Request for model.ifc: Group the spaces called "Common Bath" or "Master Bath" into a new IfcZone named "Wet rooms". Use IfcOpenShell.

First a look at what the model holds.

```python
import ifcopenshell

model = ifcopenshell.open("model.ifc")
print(model.schema)
seen = {}
for space in model.by_type("IfcSpace"):
    seen[space.LongName] = seen.get(space.LongName, 0) + 1
for name, count in sorted(seen.items(), key=str):
    print(count, "x", name)
print("zones:", [z.Name for z in model.by_type("IfcZone")][:20])
```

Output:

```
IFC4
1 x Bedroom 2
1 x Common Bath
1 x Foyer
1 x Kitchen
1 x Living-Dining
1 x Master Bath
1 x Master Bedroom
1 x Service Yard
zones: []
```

```python
import ifcopenshell
import ifcopenshell.api.group
import ifcopenshell.api.root

model = ifcopenshell.open("model.ifc")

names = {"Common Bath", "Master Bath"}
spaces = [s for s in model.by_type("IfcSpace") if s.LongName in names]

zone = ifcopenshell.api.root.create_entity(model, ifc_class="IfcZone", name="Wet rooms")
ifcopenshell.api.group.assign_group(model, products=spaces, group=zone)
print(len(spaces), "spaces in", zone.Name)

model.write("model_updated.ifc")
```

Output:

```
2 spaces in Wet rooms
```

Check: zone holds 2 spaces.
